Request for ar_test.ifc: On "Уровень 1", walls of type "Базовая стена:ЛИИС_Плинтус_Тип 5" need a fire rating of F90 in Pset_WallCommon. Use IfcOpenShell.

First a look at what the model holds.

```python
import ifcopenshell
import ifcopenshell.util.element

model = ifcopenshell.open("ar_test.ifc")
print(model.schema)
storey = next(s for s in model.by_type("IfcBuildingStorey") if s.Name == "Уровень 1")
walls = [e for e in ifcopenshell.util.element.get_decomposition(storey) if e.is_a("IfcWall")]
seen = {}
for e in walls:
    element_type = ifcopenshell.util.element.get_type(e)
    key = (element_type.Name if element_type != e and element_type else None, ifcopenshell.util.element.get_pset(e, "Pset_WallCommon", "FireRating"))
    seen[key] = seen.get(key, 0) + 1
for (name, value), count in sorted(seen.items(), key=str):
    print(count, "x", name, "|", value)
```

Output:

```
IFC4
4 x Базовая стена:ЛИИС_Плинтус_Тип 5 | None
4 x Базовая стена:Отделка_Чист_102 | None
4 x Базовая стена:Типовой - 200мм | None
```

```python
import ifcopenshell
import ifcopenshell.api.pset
import ifcopenshell.util.element

model = ifcopenshell.open("ar_test.ifc")

storey = next(s for s in model.by_type("IfcBuildingStorey") if s.Name == "Уровень 1")
walls = [e for e in ifcopenshell.util.element.get_decomposition(storey) if e.is_a("IfcWall")]

count = 0
for e in walls:
    element_type = ifcopenshell.util.element.get_type(e)
    if element_type in (None, e) or element_type.Name != "Базовая стена:ЛИИС_Плинтус_Тип 5":
        continue
    # add_pset returns the element's existing set when there is one.
    pset = ifcopenshell.api.pset.add_pset(model, product=e, name="Pset_WallCommon")
    ifcopenshell.api.pset.edit_pset(model, pset=pset, properties={"FireRating": "F90"})
    count += 1

print(count, "walls updated")

model.write("ar_test-out.ifc")
```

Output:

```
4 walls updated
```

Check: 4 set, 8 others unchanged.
